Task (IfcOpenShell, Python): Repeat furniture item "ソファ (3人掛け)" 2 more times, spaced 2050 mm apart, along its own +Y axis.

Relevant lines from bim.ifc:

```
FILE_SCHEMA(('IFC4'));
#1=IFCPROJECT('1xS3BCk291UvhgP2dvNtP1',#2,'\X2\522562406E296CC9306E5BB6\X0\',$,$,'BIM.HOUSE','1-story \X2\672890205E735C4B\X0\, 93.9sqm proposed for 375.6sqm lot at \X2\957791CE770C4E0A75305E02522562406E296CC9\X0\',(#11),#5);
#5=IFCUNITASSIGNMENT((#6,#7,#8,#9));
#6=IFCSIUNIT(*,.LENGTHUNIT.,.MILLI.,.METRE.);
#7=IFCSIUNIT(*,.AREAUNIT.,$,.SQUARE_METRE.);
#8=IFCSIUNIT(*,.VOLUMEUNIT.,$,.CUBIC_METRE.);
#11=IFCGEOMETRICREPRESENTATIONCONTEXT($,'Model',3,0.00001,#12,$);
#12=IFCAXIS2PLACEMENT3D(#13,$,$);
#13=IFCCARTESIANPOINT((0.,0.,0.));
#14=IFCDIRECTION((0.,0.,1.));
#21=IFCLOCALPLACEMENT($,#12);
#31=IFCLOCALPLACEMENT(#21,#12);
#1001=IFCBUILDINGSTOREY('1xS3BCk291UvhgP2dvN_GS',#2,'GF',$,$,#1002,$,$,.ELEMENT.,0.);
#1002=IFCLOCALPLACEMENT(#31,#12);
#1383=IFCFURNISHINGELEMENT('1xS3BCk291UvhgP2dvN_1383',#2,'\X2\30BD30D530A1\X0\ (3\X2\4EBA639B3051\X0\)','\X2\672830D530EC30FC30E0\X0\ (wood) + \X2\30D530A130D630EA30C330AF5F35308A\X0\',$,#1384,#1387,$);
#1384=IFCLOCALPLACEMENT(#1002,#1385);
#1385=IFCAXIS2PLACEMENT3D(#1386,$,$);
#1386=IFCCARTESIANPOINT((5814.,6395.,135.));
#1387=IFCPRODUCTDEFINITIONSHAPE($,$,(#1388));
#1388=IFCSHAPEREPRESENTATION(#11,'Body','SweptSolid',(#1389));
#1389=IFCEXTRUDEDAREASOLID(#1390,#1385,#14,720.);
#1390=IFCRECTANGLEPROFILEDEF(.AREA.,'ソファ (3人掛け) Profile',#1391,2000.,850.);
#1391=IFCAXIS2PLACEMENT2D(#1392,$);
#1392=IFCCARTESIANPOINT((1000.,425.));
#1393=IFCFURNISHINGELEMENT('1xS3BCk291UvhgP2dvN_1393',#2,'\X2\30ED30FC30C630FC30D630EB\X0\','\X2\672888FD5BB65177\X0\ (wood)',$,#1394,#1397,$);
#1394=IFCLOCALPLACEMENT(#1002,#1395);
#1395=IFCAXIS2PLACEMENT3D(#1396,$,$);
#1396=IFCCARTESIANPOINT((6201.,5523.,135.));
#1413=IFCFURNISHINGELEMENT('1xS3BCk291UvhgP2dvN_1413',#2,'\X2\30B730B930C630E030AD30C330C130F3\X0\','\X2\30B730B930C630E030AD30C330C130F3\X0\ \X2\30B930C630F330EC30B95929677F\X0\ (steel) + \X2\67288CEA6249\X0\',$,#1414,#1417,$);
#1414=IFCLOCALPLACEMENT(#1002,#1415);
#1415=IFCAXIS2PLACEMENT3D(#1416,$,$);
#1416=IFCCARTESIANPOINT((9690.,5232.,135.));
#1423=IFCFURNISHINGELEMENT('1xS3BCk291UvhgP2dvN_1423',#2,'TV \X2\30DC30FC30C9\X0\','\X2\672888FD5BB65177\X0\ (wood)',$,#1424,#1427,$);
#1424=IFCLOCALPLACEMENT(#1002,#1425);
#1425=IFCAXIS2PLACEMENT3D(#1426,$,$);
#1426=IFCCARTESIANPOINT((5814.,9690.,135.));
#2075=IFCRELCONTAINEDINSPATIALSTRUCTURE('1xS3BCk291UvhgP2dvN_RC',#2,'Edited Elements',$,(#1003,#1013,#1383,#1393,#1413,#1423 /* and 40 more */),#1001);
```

```python
import ifcopenshell
import ifcopenshell.api.geometry
import ifcopenshell.api.root
import ifcopenshell.util.element
import ifcopenshell.util.placement
import ifcopenshell.util.unit

model = ifcopenshell.open("bim.ifc")
unit_scale = ifcopenshell.util.unit.calculate_unit_scale(model)


def reuse_history(source, copy):
    """copy_class also copies each property set's owner history, people and application; keep the originals."""
    for rel in copy.IsDefinedBy:
        if rel.is_a("IfcRelDefinesByProperties") and (history := rel.RelatingPropertyDefinition.OwnerHistory):
            rel.RelatingPropertyDefinition.OwnerHistory = source.OwnerHistory
            ifcopenshell.util.element.remove_deep2(model, history)


source = model.by_id(1383)
base = ifcopenshell.util.placement.get_local_placement(source.ObjectPlacement)
step = base[:3, 1] * 2.05 / unit_scale

for i in range(1, 3):
    copy = ifcopenshell.api.root.copy_class(model, product=source)
    copy.Representation = ifcopenshell.util.element.copy_deep(
        model, source.Representation, exclude=["IfcGeometricRepresentationContext", "IfcRepresentationMap"]
    )
    reuse_history(source, copy)
    matrix = base.copy()
    matrix[:3, 3] += i * step
    print("added at", matrix[:3, 3].round(3) + 0.0)
    ifcopenshell.api.geometry.edit_object_placement(model, product=copy, matrix=matrix, is_si=False)

model.write("bim_rev.ifc")
```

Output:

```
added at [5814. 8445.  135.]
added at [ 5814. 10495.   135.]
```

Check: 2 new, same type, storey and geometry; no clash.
